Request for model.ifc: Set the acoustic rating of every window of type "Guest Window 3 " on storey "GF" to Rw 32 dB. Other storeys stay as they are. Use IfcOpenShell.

First a look at what the model holds.

```python
import ifcopenshell
import ifcopenshell.util.element

model = ifcopenshell.open("model.ifc")
print(model.schema)
storey = next(s for s in model.by_type("IfcBuildingStorey") if s.Name == "GF")
windows = [e for e in ifcopenshell.util.element.get_decomposition(storey) if e.is_a("IfcWindow")]
seen = {}
for e in windows:
    element_type = ifcopenshell.util.element.get_type(e)
    key = (element_type.Name if element_type != e and element_type else None, ifcopenshell.util.element.get_pset(e, "Pset_WindowCommon", "AcousticRating"))
    seen[key] = seen.get(key, 0) + 1
for (name, value), count in sorted(seen.items(), key=str):
    print(count, "x", name, "|", value)
```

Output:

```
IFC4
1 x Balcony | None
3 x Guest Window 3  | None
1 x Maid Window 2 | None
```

```python
import ifcopenshell
import ifcopenshell.api.pset
import ifcopenshell.util.element

model = ifcopenshell.open("model.ifc")

storey = next(s for s in model.by_type("IfcBuildingStorey") if s.Name == "GF")
windows = [e for e in ifcopenshell.util.element.get_decomposition(storey) if e.is_a("IfcWindow")]

count = 0
for e in windows:
    element_type = ifcopenshell.util.element.get_type(e)
    if element_type in (None, e) or element_type.Name != "Guest Window 3 ":
        continue
    # add_pset returns the element's existing set when there is one.
    pset = ifcopenshell.api.pset.add_pset(model, product=e, name="Pset_WindowCommon")
    ifcopenshell.api.pset.edit_pset(model, pset=pset, properties={"AcousticRating": "Rw 32 dB"})
    count += 1

print(count, "windows updated")

model.write("model_v2.ifc")
```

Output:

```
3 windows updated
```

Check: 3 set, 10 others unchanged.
